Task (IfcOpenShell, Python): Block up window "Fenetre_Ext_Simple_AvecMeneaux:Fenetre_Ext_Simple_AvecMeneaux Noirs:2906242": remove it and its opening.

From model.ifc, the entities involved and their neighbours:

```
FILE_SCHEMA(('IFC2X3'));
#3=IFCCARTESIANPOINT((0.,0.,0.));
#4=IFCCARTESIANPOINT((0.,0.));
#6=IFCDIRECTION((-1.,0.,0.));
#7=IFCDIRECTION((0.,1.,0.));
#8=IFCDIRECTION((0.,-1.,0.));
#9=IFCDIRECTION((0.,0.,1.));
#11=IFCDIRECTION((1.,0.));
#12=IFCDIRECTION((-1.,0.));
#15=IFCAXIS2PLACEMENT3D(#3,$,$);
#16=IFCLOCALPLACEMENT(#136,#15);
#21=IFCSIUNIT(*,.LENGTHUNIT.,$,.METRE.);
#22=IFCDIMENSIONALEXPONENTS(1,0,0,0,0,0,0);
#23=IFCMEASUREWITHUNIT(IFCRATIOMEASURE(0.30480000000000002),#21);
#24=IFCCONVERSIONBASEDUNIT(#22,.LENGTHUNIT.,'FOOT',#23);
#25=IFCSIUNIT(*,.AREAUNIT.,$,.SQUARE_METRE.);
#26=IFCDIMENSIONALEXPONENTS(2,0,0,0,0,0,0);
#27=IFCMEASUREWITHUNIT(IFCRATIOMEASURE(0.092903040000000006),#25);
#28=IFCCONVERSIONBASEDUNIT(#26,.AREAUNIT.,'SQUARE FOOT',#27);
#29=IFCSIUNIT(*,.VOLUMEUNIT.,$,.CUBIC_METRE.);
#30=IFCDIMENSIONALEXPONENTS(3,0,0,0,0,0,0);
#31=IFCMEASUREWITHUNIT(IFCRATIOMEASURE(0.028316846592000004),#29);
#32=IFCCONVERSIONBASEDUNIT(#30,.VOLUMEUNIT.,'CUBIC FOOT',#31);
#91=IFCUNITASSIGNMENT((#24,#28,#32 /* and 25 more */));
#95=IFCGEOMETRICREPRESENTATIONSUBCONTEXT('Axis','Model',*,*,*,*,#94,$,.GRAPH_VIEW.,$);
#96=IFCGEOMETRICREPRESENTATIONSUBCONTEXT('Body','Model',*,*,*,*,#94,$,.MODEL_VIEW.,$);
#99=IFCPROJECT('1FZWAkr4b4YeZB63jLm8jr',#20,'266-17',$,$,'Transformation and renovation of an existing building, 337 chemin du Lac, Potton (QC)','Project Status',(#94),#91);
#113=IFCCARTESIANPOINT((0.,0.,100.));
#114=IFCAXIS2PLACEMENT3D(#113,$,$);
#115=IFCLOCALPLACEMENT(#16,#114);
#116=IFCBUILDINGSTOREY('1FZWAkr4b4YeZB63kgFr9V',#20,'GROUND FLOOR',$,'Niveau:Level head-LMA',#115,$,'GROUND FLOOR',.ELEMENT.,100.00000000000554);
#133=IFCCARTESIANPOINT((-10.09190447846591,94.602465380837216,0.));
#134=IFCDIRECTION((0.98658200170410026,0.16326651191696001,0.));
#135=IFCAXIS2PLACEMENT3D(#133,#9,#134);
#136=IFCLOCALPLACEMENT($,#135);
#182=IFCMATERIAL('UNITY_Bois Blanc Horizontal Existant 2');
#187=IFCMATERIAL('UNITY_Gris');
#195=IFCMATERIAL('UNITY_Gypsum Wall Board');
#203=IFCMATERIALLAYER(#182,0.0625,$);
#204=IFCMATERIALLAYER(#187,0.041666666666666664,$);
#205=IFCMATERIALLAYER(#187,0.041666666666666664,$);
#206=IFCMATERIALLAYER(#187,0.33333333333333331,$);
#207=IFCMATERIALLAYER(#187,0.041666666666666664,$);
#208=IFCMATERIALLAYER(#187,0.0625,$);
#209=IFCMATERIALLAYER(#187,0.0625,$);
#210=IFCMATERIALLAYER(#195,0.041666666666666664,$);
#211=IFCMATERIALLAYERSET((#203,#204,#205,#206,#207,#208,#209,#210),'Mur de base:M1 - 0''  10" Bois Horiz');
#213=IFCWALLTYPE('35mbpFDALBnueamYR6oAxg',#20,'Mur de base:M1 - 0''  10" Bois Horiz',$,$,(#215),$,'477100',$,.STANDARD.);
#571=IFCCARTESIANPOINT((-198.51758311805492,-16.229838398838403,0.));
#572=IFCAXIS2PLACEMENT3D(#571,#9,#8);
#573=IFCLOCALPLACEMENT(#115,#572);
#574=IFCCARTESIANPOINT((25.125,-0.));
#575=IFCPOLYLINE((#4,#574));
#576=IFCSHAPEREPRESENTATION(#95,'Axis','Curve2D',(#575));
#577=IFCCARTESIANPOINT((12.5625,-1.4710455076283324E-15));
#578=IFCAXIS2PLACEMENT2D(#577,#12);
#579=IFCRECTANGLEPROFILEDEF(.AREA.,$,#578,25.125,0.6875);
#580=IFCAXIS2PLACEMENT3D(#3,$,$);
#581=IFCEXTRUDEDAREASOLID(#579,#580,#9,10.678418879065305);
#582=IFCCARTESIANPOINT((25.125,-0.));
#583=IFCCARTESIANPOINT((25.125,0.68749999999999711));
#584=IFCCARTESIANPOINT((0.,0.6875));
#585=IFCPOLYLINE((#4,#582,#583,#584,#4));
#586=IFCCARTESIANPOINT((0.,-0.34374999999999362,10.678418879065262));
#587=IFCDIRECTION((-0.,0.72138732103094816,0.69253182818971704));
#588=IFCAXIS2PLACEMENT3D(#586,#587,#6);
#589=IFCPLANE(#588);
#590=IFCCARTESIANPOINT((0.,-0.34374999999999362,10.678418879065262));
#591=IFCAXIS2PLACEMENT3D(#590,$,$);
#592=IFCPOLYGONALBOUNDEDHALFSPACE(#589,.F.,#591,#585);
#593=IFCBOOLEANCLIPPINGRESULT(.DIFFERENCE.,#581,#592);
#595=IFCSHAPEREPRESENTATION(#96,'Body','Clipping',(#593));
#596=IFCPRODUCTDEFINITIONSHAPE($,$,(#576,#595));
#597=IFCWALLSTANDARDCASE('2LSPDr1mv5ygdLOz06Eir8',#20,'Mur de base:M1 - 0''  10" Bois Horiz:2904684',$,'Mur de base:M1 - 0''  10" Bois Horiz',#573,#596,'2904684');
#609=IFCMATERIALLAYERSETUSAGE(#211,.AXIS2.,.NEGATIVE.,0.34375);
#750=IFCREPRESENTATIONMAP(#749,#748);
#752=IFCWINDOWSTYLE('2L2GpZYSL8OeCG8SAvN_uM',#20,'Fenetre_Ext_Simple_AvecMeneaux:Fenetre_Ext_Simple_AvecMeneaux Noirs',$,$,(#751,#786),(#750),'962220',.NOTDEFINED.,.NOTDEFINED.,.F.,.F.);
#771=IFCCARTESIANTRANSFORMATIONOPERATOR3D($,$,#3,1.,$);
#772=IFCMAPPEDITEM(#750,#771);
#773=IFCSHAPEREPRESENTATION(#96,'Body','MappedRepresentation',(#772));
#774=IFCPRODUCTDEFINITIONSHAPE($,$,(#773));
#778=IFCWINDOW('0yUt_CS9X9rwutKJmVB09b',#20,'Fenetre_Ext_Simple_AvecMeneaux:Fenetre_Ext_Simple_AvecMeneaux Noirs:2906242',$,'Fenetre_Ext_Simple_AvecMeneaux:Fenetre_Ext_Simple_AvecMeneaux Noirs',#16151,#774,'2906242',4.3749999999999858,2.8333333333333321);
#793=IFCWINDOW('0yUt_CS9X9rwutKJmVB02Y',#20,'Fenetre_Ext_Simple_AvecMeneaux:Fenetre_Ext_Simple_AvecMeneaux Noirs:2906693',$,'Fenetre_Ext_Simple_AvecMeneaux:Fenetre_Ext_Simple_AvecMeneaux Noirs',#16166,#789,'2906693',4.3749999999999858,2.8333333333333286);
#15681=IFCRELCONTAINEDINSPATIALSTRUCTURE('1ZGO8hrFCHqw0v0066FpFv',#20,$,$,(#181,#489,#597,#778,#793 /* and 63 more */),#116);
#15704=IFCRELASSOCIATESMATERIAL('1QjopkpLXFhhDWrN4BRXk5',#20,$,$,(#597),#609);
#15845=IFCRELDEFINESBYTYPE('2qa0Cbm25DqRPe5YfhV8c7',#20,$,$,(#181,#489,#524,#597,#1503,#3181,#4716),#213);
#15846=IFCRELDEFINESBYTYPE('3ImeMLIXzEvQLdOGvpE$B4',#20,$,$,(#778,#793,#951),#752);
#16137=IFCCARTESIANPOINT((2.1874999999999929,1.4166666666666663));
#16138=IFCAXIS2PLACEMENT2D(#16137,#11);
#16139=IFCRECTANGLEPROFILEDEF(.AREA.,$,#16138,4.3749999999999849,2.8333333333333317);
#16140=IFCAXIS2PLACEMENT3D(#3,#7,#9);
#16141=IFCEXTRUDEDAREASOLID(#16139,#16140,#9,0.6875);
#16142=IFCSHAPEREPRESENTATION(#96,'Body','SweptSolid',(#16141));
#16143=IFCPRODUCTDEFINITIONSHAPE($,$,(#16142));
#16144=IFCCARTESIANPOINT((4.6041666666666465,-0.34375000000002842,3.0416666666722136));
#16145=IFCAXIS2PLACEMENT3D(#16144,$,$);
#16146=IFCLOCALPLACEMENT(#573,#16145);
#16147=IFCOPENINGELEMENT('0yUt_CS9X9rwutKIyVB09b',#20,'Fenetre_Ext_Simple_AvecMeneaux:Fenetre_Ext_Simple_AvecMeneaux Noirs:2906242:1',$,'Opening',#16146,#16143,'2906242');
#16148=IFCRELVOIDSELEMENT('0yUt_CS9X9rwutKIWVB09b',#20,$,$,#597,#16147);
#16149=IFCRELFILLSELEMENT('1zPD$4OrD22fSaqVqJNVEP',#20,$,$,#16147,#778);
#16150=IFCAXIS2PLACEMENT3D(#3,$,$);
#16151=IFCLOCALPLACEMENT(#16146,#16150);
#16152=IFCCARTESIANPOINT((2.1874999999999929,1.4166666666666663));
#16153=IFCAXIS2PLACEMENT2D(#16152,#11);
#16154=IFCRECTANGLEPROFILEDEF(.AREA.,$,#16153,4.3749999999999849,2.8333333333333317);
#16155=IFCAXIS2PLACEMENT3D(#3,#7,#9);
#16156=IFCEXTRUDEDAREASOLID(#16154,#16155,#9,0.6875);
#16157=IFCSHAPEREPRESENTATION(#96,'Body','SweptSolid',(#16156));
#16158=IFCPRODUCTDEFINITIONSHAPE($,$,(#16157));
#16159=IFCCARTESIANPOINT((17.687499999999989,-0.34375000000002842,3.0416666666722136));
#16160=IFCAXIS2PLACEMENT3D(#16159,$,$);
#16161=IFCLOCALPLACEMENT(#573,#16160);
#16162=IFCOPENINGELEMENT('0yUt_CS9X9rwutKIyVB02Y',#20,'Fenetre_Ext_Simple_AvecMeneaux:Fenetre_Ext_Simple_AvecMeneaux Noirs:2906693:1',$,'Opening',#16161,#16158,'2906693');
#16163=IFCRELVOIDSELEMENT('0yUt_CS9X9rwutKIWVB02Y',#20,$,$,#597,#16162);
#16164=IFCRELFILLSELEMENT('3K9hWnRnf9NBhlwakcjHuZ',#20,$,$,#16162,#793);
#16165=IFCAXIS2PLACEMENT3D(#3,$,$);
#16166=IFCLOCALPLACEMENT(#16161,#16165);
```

```python
import ifcopenshell
import ifcopenshell.api.feature
import ifcopenshell.api.root
import ifcopenshell.geom
import ifcopenshell.util.shape

model = ifcopenshell.open("model.ifc")
settings = ifcopenshell.geom.settings()


def volume(element):
    """Net volume in cubic metres, openings subtracted."""
    shape = ifcopenshell.geom.create_shape(settings, element)
    return ifcopenshell.util.shape.get_volume(shape.geometry)


window = model.by_guid("0yUt_CS9X9rwutKJmVB09b")
opening = window.FillsVoids[0].RelatingOpeningElement
wall = opening.VoidsElements[0].RelatingBuildingElement
before = volume(wall)

ifcopenshell.api.root.remove_product(model, product=window)
ifcopenshell.api.feature.remove_feature(model, feature=opening)

after = volume(wall)

print(f"wall volume {before:.3f} -> {after:.3f} m3")

model.write("model_updated.ifc")
```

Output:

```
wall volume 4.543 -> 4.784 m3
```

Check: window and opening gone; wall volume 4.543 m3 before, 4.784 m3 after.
